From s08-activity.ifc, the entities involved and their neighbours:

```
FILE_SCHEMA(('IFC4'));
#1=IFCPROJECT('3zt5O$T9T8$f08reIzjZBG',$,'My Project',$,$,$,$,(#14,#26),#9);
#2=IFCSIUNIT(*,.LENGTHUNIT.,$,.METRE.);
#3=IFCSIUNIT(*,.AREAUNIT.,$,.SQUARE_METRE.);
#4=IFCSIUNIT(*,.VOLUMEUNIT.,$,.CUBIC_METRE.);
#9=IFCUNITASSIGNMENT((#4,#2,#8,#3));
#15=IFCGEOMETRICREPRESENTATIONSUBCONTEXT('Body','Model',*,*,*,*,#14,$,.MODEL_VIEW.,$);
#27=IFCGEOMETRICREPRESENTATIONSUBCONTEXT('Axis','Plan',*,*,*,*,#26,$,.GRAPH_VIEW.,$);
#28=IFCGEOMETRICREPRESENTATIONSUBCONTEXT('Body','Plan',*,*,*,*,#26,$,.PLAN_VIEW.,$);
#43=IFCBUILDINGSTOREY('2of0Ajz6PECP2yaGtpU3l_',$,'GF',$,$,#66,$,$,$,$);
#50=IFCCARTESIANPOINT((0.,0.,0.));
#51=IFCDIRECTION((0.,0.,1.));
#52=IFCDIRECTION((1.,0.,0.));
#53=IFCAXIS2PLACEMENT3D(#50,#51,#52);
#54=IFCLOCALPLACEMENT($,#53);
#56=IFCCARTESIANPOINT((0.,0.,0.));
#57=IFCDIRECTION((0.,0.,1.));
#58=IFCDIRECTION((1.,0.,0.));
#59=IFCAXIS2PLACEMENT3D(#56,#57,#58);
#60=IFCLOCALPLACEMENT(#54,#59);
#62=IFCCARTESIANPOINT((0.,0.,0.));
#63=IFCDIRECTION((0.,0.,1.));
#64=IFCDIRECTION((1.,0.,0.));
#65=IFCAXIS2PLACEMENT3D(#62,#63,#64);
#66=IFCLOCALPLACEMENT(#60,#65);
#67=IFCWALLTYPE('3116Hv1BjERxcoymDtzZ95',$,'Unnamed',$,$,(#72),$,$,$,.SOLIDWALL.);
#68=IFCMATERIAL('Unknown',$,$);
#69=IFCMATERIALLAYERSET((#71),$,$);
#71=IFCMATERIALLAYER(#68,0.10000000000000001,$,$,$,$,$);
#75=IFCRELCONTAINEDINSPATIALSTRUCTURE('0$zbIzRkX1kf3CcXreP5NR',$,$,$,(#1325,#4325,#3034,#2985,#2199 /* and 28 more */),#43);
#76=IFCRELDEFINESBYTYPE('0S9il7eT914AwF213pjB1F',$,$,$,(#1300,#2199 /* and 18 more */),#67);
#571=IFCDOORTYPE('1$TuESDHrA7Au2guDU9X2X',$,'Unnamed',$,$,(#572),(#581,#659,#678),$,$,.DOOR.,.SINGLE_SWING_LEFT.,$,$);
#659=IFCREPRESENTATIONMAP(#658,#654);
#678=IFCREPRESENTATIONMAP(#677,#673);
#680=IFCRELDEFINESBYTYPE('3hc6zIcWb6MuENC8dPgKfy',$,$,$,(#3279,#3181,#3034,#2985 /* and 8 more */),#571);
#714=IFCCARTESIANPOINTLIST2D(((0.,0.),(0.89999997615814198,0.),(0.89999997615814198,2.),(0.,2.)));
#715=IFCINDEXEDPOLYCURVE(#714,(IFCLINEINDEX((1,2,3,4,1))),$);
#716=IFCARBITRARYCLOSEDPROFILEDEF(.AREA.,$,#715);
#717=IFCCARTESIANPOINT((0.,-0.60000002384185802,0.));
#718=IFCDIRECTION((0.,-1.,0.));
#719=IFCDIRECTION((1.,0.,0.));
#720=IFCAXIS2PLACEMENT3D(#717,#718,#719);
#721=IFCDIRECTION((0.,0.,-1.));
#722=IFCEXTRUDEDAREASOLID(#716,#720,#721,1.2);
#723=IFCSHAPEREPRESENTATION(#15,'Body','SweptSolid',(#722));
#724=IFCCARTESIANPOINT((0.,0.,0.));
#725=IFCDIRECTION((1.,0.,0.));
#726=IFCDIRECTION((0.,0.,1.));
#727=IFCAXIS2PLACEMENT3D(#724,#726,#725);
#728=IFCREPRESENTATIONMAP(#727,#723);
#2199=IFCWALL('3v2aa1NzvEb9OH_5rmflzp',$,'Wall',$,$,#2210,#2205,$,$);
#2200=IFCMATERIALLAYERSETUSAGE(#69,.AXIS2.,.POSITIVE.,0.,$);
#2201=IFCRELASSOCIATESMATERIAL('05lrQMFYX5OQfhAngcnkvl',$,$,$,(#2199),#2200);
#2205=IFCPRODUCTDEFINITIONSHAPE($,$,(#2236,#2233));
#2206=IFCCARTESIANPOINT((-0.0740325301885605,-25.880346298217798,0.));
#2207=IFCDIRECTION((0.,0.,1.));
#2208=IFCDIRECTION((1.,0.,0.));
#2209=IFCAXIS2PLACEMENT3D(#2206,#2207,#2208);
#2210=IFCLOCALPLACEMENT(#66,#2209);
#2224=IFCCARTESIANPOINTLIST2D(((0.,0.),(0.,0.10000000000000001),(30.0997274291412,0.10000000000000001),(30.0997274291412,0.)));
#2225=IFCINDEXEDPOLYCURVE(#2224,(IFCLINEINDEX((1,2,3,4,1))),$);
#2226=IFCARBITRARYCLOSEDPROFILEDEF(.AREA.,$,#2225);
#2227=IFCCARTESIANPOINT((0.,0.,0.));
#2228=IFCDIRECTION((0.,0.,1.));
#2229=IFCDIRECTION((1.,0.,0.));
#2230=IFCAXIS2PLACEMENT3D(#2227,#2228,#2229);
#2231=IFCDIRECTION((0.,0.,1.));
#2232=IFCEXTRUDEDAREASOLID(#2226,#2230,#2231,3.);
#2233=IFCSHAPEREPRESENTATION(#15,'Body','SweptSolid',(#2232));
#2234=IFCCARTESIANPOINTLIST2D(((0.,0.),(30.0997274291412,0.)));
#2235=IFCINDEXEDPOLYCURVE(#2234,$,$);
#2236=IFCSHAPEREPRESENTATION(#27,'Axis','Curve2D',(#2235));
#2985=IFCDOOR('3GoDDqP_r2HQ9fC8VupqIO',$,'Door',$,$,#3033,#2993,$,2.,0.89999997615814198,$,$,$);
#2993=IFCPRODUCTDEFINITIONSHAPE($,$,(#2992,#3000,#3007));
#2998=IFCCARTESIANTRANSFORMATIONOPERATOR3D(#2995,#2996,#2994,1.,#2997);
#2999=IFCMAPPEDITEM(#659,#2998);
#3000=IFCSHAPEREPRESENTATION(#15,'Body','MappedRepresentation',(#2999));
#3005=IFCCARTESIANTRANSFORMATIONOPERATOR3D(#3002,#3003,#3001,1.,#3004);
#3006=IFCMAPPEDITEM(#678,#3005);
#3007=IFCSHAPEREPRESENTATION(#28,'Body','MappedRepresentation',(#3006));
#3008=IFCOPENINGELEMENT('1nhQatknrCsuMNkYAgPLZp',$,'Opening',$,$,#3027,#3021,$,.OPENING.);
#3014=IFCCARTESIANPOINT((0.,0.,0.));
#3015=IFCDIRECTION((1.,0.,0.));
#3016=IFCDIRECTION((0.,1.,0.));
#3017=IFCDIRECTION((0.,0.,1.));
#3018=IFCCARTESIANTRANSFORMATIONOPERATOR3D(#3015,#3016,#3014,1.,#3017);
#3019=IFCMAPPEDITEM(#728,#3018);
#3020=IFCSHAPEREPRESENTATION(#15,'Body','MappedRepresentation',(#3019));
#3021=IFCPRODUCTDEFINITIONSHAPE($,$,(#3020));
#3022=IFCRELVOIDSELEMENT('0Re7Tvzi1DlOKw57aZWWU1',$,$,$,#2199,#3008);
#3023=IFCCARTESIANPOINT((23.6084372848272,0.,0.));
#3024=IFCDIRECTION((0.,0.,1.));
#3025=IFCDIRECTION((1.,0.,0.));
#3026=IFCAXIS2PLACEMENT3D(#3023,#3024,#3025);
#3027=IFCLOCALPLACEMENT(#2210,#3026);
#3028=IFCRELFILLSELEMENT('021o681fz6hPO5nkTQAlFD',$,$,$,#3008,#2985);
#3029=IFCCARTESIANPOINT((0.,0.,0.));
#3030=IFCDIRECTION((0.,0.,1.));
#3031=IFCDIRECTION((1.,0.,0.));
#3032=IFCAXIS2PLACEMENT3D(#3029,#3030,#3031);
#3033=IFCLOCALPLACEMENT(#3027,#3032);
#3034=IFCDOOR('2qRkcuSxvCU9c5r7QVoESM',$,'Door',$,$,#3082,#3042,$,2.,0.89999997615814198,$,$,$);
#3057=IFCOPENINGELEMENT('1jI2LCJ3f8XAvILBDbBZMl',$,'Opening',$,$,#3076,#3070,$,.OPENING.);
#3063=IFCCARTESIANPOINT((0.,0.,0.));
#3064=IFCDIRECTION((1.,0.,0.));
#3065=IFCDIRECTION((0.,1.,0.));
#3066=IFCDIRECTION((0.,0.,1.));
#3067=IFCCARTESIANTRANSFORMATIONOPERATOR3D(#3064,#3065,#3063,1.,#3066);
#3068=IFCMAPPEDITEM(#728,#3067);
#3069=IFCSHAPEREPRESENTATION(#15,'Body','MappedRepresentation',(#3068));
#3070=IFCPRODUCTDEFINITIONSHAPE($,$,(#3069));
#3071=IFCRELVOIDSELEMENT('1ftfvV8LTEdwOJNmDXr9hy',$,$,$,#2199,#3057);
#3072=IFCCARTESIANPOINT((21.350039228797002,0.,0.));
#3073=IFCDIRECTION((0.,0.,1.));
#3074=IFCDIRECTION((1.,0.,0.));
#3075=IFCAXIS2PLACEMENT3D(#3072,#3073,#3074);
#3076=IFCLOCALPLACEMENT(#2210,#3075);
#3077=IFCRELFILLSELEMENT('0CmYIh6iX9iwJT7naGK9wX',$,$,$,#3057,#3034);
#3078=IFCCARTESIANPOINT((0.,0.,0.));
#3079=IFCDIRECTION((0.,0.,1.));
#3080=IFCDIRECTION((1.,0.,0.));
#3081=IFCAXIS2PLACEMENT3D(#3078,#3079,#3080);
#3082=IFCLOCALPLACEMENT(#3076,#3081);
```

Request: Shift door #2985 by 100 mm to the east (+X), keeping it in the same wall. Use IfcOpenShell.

```python
import ifcopenshell
import ifcopenshell.api.geometry
import ifcopenshell.util.placement

model = ifcopenshell.open("s08-activity.ifc")

door = model.by_id(2985)
opening = door.FillsVoids[0].RelatingOpeningElement
wall = opening.VoidsElements[0].RelatingBuildingElement

wall_matrix = ifcopenshell.util.placement.get_local_placement(wall.ObjectPlacement)
shift = wall_matrix[:3, 0] * 0.1
before = ifcopenshell.util.placement.get_local_placement(door.ObjectPlacement)[:3, 3].copy()

# The door is placed relative to its opening, so it follows when the opening moves.
matrix = ifcopenshell.util.placement.get_local_placement(opening.ObjectPlacement)
matrix[:3, 3] += shift
ifcopenshell.api.geometry.edit_object_placement(
    model, product=opening, matrix=matrix, is_si=False, should_transform_children=True
)

after = ifcopenshell.util.placement.get_local_placement(door.ObjectPlacement)[:3, 3]
print("door moved by", (after - before).round(3) + 0.0)

model.write("s08-activity_updated.ifc")
```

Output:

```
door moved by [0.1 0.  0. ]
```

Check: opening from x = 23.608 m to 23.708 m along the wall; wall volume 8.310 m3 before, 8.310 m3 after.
